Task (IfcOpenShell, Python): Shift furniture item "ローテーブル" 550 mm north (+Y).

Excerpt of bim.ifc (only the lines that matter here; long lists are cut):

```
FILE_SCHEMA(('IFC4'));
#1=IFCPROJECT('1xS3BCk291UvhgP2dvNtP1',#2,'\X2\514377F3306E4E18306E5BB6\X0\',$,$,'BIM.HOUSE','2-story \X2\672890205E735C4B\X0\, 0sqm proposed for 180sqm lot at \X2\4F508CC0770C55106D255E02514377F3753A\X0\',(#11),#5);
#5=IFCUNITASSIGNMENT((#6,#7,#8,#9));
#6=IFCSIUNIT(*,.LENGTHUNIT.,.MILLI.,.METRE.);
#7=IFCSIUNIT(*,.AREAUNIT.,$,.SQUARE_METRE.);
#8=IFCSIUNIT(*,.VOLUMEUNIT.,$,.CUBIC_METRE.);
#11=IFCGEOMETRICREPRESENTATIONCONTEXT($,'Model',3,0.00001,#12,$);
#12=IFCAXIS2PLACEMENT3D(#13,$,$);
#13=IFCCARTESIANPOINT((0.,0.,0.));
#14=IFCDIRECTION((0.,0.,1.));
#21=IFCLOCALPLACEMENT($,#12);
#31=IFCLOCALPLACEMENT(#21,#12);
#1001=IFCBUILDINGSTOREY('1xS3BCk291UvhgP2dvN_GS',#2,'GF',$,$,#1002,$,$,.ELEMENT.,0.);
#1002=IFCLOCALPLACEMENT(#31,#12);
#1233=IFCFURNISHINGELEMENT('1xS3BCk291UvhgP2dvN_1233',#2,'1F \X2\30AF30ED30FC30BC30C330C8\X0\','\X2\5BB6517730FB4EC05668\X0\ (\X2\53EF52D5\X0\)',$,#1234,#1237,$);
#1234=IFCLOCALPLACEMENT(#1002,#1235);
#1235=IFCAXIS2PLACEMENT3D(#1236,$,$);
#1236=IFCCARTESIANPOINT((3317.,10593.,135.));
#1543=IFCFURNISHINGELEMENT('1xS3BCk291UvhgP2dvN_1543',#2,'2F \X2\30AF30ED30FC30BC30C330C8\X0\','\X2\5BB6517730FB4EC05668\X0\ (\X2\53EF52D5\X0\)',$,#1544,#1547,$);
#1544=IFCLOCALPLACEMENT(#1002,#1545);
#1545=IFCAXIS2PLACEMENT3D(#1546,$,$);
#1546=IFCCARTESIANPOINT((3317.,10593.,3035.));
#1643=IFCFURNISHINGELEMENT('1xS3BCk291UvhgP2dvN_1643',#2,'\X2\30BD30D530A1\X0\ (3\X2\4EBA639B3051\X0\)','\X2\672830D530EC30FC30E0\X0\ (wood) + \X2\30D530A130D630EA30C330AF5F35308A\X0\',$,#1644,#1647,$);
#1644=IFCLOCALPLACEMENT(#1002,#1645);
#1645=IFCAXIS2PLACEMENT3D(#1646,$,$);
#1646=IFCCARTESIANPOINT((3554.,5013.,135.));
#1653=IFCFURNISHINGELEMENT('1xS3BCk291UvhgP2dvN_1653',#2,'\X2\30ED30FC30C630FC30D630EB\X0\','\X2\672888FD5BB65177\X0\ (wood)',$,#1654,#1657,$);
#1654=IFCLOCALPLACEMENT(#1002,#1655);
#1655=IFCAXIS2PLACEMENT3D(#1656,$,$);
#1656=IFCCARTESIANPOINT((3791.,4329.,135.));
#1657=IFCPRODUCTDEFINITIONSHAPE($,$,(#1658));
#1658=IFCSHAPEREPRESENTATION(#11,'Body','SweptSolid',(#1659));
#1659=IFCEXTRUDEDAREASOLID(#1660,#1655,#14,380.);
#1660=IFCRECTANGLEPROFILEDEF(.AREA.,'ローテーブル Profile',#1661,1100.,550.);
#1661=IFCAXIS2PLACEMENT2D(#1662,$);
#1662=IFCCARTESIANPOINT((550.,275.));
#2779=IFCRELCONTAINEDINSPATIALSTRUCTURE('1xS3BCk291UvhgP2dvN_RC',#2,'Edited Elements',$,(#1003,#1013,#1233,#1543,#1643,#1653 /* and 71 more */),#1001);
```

```python
import ifcopenshell
import ifcopenshell.api.geometry
import ifcopenshell.util.placement

model = ifcopenshell.open("bim.ifc")

item = model.by_guid("1xS3BCk291UvhgP2dvN_1653")
matrix = ifcopenshell.util.placement.get_local_placement(item.ObjectPlacement)
matrix[1, 3] += 550.0
ifcopenshell.api.geometry.edit_object_placement(model, product=item, matrix=matrix, is_si=False)

print(ifcopenshell.util.placement.get_local_placement(item.ObjectPlacement).round(3) + 0.0)

model.write("bim_rev.ifc")
```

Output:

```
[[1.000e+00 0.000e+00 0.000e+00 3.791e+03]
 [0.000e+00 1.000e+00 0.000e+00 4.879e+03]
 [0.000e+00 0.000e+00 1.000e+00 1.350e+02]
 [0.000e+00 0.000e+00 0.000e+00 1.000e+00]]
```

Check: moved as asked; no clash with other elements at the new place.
